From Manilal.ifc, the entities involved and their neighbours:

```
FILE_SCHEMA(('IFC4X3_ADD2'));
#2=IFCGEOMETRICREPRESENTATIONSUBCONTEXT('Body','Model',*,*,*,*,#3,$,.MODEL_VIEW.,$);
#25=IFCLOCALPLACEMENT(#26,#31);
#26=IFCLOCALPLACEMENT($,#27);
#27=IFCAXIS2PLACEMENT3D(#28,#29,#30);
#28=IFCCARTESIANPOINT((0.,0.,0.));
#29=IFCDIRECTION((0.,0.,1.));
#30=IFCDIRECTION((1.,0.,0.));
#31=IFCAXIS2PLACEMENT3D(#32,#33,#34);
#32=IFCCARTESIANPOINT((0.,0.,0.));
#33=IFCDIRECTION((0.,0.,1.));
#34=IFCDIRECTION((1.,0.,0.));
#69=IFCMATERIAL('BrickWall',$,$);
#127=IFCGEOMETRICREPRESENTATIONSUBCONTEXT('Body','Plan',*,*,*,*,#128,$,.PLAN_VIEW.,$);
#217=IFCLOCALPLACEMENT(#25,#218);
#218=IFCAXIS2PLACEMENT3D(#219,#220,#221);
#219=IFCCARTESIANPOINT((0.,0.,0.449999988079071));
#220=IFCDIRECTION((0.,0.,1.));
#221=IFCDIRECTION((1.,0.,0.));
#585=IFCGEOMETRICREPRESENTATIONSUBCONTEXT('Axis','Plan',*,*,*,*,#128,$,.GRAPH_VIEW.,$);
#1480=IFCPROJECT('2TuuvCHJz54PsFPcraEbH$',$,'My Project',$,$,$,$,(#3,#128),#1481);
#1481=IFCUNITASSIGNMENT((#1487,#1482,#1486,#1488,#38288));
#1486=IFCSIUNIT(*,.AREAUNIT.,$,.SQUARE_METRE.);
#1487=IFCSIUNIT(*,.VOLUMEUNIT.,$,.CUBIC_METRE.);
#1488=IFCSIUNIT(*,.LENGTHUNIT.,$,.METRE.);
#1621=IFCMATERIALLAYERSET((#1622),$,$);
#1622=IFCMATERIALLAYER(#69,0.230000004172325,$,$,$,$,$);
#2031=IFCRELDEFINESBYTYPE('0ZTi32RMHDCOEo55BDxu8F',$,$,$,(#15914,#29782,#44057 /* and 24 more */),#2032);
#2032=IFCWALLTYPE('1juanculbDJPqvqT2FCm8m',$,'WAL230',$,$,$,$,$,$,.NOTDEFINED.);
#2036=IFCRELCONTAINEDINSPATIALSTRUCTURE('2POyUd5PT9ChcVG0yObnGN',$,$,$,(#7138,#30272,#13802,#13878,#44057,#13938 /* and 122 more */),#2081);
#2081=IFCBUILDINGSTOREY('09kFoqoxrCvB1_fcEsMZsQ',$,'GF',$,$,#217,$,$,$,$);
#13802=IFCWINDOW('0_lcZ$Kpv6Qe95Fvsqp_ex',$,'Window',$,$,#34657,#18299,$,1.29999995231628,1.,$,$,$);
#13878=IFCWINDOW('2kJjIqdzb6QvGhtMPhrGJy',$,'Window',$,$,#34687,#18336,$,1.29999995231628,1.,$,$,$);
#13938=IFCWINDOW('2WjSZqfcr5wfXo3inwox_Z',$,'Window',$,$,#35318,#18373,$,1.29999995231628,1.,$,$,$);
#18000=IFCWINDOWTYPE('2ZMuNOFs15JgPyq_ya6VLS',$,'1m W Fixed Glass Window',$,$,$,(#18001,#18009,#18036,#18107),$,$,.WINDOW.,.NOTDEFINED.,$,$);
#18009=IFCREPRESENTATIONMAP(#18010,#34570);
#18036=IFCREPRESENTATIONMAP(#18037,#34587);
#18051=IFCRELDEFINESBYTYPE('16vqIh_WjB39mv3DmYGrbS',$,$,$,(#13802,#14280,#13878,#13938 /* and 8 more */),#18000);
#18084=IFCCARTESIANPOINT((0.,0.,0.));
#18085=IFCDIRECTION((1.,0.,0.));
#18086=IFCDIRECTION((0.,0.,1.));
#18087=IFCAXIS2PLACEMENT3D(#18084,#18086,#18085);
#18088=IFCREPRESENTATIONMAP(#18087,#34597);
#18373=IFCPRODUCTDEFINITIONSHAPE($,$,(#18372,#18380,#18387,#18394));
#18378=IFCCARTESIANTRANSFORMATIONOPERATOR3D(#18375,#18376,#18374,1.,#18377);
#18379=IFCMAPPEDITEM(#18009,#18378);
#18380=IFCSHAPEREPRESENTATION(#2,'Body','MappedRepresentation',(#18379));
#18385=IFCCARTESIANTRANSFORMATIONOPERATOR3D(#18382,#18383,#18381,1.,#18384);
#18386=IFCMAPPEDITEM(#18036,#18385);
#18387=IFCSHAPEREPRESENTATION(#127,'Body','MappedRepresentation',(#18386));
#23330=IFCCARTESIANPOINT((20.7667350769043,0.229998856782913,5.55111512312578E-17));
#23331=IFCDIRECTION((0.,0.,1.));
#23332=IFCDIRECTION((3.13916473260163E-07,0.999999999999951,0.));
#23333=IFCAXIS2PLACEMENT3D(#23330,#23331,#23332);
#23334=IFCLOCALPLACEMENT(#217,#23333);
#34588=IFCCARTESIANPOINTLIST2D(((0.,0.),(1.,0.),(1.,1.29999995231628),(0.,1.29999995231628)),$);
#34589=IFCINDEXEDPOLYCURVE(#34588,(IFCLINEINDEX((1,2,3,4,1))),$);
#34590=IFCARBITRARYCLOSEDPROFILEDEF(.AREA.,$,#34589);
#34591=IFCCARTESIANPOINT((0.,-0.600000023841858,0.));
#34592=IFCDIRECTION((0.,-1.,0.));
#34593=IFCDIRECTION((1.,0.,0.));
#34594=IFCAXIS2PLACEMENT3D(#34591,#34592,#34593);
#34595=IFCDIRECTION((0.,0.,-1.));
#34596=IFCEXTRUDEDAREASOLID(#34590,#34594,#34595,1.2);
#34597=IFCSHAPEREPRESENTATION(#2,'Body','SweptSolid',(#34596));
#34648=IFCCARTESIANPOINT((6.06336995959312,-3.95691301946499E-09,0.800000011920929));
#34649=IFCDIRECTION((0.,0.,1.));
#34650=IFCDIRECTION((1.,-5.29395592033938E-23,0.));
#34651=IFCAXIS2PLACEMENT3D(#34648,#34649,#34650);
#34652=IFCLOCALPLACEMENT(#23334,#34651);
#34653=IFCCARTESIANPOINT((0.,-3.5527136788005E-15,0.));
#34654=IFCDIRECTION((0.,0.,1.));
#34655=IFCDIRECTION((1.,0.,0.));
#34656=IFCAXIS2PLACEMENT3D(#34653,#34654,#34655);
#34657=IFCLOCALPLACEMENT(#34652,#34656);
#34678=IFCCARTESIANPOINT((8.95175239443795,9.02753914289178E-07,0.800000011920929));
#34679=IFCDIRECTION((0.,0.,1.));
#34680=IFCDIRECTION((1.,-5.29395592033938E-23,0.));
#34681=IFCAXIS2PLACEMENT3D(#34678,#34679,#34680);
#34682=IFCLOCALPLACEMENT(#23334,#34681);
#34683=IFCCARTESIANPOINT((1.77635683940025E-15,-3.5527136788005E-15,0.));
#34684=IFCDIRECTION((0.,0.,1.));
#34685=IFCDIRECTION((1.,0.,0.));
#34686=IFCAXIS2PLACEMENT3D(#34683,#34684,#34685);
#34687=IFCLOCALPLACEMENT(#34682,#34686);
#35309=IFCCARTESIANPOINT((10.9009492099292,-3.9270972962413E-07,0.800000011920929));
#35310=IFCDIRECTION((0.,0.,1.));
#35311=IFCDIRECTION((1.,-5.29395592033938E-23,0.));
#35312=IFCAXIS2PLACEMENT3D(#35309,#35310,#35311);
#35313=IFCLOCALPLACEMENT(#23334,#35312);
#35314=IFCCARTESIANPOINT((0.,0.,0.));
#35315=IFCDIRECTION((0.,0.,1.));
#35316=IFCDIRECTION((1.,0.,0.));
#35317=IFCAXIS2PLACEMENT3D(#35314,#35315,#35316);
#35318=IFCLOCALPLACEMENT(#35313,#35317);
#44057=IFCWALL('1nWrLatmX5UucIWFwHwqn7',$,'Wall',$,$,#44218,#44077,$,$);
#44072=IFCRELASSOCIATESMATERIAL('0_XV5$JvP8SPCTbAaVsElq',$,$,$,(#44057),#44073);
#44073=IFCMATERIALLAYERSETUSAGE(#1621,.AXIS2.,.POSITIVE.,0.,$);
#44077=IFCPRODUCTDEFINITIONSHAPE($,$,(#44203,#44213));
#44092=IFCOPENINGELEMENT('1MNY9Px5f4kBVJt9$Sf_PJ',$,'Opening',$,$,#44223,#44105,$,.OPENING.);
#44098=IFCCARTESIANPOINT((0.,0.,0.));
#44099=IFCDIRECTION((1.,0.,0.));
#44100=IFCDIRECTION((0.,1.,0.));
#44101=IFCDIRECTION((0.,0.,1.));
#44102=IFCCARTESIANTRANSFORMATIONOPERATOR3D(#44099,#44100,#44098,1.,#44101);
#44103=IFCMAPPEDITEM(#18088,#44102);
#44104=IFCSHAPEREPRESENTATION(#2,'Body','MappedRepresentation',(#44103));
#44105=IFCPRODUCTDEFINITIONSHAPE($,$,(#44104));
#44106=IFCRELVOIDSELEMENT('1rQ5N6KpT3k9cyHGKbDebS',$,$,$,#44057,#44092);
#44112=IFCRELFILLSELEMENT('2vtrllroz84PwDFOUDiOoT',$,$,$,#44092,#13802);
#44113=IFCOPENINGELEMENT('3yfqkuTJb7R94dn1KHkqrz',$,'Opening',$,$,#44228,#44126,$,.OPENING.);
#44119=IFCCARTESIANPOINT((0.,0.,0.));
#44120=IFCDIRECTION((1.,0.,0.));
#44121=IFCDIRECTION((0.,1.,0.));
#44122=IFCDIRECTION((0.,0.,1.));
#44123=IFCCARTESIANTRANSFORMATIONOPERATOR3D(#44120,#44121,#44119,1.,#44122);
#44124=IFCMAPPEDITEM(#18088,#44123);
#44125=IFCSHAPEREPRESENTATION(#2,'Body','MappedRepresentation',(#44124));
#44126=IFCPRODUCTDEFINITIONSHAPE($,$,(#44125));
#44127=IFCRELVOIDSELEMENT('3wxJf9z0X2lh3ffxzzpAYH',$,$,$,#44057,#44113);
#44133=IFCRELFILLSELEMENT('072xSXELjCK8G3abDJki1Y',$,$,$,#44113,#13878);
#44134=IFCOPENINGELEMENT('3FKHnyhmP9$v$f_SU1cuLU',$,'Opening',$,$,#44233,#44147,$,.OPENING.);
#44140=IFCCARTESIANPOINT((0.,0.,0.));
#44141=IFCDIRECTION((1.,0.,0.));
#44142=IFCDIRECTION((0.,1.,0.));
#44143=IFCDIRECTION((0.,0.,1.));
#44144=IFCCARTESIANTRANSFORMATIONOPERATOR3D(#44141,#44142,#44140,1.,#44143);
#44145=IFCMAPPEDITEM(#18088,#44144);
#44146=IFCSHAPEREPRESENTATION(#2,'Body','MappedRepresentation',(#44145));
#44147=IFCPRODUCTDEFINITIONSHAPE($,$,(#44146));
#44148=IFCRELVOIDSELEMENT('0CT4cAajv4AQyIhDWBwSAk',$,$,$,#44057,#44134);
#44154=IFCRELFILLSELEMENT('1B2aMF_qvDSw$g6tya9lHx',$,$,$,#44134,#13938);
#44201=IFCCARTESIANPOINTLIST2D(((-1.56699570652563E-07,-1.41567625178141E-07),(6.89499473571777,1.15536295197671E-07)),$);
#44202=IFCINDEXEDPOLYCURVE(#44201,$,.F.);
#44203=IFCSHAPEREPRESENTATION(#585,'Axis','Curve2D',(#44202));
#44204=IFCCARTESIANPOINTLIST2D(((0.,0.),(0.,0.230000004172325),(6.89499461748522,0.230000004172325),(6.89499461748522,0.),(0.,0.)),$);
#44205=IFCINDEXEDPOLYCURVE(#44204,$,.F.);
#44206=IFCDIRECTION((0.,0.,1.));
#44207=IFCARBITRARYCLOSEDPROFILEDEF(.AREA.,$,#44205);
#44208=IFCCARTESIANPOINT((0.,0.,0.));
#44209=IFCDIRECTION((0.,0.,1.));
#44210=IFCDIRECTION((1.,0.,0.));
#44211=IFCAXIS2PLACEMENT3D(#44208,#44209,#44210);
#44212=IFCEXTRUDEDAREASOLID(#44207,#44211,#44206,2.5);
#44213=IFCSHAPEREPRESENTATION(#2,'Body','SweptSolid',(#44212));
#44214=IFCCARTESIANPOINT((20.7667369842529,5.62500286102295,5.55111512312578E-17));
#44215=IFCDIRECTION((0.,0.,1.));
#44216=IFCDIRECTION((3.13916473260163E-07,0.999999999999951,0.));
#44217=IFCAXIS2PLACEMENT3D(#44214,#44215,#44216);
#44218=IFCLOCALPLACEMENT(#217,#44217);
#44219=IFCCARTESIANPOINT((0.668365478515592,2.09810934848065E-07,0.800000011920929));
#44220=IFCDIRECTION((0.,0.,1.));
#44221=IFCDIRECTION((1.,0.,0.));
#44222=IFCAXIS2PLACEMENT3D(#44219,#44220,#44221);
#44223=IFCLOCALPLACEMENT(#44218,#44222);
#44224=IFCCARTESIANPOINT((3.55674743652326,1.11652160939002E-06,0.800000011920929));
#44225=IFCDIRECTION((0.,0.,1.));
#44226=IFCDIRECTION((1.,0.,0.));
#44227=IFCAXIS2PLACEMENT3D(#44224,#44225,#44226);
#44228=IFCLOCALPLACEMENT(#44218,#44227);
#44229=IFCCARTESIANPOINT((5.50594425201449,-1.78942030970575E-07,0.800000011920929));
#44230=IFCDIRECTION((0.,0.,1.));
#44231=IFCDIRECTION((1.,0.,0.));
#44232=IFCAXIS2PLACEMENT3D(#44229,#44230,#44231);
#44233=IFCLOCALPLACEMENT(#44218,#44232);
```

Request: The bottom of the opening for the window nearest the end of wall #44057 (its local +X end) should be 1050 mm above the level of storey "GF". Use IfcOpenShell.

```python
import numpy as np
import ifcopenshell
import ifcopenshell.api.geometry
import ifcopenshell.geom
import ifcopenshell.util.element
import ifcopenshell.util.placement
import ifcopenshell.util.shape
import ifcopenshell.util.unit

model = ifcopenshell.open("Manilal.ifc")
unit_scale = ifcopenshell.util.unit.calculate_unit_scale(model)

window = model.by_id(13938)
opening = window.FillsVoids[0].RelatingOpeningElement
storey = ifcopenshell.util.element.get_container(window, ifc_class="IfcBuildingStorey")
level = ifcopenshell.util.placement.get_local_placement(storey.ObjectPlacement)[2, 3]

# The opening's origin need not be at the sill, so measure its lowest point.
shape = ifcopenshell.geom.create_shape(ifcopenshell.geom.settings(), opening)
bottom = ifcopenshell.util.shape.get_shape_bottom_elevation(shape, shape.geometry) / unit_scale
dz = level + 1.05 / unit_scale - bottom

shift = np.array([0.0, 0.0, dz])
# The window is not placed relative to its opening, so move both.
for product in (opening, window):
    matrix = ifcopenshell.util.placement.get_local_placement(product.ObjectPlacement)
    matrix[:3, 3] += shift
    ifcopenshell.api.geometry.edit_object_placement(model, product=product, matrix=matrix, is_si=False)

print(f"moved by {dz * unit_scale:+.3f} m")

model.write("Manilal_edited.ifc")
```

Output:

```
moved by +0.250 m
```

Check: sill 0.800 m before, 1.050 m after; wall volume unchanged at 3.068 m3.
